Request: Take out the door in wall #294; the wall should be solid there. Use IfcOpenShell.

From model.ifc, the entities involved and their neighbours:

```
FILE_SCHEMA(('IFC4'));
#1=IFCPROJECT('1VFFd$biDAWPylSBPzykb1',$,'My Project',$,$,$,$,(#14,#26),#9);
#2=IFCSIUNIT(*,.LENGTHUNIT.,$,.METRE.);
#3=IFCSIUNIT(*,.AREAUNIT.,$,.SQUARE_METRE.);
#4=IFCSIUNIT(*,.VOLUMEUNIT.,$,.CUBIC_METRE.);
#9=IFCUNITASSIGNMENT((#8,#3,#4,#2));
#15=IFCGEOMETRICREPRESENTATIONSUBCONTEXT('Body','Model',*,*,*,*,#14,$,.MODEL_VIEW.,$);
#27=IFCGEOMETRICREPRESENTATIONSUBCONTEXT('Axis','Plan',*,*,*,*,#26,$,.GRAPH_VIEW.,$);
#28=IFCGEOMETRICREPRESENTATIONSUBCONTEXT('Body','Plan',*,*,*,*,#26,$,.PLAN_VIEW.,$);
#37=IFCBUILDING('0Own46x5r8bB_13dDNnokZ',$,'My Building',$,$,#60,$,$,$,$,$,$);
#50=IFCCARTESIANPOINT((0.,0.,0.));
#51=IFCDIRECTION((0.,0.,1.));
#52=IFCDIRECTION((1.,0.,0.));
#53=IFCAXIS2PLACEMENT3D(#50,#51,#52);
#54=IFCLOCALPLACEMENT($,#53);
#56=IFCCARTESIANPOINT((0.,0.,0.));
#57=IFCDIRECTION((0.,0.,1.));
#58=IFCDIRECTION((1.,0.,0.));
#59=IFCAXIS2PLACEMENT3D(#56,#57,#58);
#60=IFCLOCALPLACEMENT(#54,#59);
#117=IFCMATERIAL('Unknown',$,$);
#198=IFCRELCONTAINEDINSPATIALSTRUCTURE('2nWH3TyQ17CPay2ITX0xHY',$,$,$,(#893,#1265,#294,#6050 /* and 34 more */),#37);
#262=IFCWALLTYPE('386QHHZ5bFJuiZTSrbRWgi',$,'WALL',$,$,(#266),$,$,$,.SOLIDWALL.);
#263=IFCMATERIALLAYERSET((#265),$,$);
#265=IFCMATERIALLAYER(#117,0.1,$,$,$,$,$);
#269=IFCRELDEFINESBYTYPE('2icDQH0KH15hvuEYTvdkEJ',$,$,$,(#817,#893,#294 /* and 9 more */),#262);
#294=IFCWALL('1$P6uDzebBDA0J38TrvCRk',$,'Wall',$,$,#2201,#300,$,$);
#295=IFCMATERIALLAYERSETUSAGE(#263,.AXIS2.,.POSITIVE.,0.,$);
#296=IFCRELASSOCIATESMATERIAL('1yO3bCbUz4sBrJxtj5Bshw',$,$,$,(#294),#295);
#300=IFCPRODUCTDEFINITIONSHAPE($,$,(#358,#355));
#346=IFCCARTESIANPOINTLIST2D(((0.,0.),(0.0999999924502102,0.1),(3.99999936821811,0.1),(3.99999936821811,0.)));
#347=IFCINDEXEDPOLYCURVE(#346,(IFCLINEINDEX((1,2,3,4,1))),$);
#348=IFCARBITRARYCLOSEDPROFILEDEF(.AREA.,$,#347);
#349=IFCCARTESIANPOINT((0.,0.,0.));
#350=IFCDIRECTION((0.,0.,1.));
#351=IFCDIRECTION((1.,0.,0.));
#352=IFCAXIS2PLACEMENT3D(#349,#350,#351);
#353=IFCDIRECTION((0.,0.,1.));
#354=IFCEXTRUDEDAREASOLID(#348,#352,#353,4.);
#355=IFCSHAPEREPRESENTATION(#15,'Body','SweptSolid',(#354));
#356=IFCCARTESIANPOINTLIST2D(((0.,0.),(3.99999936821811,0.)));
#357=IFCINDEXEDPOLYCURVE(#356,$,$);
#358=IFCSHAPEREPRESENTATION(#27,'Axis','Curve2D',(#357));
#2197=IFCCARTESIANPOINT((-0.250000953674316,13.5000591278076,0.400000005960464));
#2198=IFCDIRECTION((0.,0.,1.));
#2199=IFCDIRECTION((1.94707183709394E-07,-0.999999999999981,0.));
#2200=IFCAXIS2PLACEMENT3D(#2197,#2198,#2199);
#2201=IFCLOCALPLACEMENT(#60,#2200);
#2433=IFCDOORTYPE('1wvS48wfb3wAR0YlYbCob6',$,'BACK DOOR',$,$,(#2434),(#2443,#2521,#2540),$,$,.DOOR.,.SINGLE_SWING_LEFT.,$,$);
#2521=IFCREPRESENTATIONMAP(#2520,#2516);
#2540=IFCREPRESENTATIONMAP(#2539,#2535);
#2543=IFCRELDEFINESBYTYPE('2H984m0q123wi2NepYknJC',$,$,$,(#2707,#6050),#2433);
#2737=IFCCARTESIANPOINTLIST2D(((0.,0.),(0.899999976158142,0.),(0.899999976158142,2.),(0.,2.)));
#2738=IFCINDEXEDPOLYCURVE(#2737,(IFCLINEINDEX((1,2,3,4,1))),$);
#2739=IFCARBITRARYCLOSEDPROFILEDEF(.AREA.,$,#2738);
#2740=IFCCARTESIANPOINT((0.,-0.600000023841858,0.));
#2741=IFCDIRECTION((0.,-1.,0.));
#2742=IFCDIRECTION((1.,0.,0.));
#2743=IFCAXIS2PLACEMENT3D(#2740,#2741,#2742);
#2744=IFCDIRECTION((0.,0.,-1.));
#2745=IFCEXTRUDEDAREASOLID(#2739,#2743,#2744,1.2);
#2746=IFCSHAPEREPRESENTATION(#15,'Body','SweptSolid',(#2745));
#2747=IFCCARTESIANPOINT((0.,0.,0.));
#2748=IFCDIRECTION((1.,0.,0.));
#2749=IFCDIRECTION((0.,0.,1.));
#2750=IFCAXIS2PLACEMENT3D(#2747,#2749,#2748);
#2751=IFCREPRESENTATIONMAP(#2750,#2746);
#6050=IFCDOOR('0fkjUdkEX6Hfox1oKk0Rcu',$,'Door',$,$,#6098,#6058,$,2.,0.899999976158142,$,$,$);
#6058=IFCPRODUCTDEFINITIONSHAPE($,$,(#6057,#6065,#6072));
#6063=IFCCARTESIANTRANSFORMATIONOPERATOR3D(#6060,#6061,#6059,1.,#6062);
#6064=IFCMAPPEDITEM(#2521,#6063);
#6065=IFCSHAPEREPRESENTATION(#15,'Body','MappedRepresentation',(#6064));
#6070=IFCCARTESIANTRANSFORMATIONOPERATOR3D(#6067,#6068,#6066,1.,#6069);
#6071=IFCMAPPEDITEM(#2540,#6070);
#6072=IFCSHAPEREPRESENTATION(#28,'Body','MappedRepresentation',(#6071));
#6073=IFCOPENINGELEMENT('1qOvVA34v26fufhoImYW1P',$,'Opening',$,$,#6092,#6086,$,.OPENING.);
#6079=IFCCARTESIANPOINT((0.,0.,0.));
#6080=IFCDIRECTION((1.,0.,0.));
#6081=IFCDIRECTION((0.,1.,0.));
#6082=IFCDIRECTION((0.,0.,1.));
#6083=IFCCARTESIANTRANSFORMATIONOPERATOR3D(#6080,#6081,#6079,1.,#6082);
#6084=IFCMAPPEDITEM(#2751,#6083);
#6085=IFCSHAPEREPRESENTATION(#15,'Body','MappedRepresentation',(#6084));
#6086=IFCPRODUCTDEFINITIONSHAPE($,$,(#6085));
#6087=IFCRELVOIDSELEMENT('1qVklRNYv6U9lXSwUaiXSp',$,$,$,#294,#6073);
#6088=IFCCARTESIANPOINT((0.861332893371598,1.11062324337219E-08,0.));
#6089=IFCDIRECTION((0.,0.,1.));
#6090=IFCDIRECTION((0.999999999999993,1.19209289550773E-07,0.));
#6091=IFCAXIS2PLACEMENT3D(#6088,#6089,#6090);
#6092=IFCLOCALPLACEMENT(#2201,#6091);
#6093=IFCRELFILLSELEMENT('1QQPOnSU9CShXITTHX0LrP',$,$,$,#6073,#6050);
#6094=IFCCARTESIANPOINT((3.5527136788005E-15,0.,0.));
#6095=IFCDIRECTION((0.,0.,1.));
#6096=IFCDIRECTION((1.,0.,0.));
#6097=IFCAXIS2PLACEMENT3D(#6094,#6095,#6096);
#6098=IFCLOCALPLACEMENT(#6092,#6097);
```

```python
import ifcopenshell
import ifcopenshell.api.feature
import ifcopenshell.api.root
import ifcopenshell.geom
import ifcopenshell.util.shape

model = ifcopenshell.open("model.ifc")
settings = ifcopenshell.geom.settings()


def volume(element):
    """Net volume in cubic metres, openings subtracted."""
    shape = ifcopenshell.geom.create_shape(settings, element)
    return ifcopenshell.util.shape.get_volume(shape.geometry)


door = model.by_guid("0fkjUdkEX6Hfox1oKk0Rcu")
opening = door.FillsVoids[0].RelatingOpeningElement
wall = opening.VoidsElements[0].RelatingBuildingElement
before = volume(wall)

ifcopenshell.api.root.remove_product(model, product=door)
ifcopenshell.api.feature.remove_feature(model, feature=opening)

after = volume(wall)

print(f"wall volume {before:.3f} -> {after:.3f} m3")

model.write("model_v2.ifc")
```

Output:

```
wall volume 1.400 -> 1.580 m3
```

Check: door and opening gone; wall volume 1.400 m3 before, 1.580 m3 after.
